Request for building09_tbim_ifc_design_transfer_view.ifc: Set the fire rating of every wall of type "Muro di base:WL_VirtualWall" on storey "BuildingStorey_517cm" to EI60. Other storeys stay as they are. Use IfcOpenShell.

First a look at what the model holds.

```python
import ifcopenshell
import ifcopenshell.util.element

model = ifcopenshell.open("building09_tbim_ifc_design_transfer_view.ifc")
print(model.schema)
storey = next(s for s in model.by_type("IfcBuildingStorey") if s.Name == "BuildingStorey_517cm")
walls = [e for e in ifcopenshell.util.element.get_decomposition(storey) if e.is_a("IfcWall")]
seen = {}
for e in walls:
    element_type = ifcopenshell.util.element.get_type(e)
    key = (element_type.Name if element_type != e and element_type else None, ifcopenshell.util.element.get_pset(e, "Pset_WallCommon", "FireRating"))
    seen[key] = seen.get(key, 0) + 1
for (name, value), count in sorted(seen.items(), key=str):
    print(count, "x", name, "|", value)
```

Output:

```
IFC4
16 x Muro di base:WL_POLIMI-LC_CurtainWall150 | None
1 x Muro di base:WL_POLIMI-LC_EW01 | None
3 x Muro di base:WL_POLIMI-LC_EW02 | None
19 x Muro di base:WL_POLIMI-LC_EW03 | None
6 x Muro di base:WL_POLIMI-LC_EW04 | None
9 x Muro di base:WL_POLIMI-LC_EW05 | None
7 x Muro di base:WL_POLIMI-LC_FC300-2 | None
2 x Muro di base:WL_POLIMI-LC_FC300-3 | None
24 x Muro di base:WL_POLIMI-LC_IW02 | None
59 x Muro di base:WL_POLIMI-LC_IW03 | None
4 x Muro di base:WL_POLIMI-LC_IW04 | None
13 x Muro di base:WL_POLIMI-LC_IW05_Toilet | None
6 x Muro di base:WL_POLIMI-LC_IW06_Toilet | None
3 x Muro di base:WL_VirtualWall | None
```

```python
import ifcopenshell
import ifcopenshell.api.pset
import ifcopenshell.util.element

model = ifcopenshell.open("building09_tbim_ifc_design_transfer_view.ifc")

storey = next(s for s in model.by_type("IfcBuildingStorey") if s.Name == "BuildingStorey_517cm")
walls = [e for e in ifcopenshell.util.element.get_decomposition(storey) if e.is_a("IfcWall")]

count = 0
for e in walls:
    element_type = ifcopenshell.util.element.get_type(e)
    if element_type in (None, e) or element_type.Name != "Muro di base:WL_VirtualWall":
        continue
    # add_pset returns the element's existing set when there is one.
    pset = ifcopenshell.api.pset.add_pset(model, product=e, name="Pset_WallCommon")
    ifcopenshell.api.pset.edit_pset(model, pset=pset, properties={"FireRating": "EI60"})
    count += 1

print(count, "walls updated")

model.write("building09_tbim_ifc_design_transfer_view-out.ifc")
```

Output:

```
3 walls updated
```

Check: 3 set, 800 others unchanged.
